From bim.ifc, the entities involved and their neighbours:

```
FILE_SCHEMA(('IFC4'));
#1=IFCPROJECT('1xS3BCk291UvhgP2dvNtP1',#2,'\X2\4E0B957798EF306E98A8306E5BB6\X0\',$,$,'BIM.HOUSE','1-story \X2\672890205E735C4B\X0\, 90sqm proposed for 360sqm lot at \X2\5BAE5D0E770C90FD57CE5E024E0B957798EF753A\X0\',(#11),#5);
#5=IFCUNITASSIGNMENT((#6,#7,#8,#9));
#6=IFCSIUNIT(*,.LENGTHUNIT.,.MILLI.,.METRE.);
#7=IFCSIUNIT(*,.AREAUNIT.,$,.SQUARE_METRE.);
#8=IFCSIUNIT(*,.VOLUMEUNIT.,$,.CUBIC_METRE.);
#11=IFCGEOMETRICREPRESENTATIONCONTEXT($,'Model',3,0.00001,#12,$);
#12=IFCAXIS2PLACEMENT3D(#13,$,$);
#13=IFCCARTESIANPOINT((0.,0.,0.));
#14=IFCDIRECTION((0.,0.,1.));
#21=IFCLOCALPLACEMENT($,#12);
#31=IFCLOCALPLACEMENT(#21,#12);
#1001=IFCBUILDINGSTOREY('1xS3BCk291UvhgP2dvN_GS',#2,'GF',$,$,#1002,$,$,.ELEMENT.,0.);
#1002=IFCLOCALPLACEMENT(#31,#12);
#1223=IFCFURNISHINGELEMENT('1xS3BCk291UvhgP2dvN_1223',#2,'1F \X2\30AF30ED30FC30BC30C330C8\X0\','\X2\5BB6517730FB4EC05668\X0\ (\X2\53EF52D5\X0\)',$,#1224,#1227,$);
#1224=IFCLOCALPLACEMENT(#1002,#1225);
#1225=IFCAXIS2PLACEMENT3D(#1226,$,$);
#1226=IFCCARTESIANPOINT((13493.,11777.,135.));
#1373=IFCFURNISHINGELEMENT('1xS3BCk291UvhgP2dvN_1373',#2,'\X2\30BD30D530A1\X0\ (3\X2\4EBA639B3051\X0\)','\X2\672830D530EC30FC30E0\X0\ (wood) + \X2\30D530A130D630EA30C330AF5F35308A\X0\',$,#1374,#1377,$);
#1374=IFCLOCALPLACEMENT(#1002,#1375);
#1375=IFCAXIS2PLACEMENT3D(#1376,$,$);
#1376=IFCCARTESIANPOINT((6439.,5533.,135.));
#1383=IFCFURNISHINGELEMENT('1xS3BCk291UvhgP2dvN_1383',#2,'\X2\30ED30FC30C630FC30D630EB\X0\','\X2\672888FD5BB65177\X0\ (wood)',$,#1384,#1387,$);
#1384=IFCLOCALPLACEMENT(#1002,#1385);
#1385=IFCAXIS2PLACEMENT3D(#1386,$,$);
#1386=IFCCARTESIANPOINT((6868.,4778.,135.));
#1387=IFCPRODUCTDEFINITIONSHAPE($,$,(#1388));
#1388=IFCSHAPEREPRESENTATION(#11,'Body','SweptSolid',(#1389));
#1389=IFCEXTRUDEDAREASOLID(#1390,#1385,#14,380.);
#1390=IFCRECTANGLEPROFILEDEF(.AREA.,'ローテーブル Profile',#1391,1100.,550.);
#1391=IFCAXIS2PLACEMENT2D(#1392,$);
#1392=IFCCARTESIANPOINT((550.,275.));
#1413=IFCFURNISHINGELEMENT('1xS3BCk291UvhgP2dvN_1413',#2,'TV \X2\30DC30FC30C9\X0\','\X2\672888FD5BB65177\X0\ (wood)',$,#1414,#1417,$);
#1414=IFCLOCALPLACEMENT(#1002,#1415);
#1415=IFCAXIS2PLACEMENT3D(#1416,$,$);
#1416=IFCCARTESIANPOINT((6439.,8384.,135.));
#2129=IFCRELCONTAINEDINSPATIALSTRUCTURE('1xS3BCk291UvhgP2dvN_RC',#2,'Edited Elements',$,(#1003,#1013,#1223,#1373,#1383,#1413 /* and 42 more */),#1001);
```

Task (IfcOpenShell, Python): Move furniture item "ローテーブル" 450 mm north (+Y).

```python
import ifcopenshell
import ifcopenshell.api.geometry
import ifcopenshell.util.placement
import ifcopenshell.util.unit

model = ifcopenshell.open("bim.ifc")
unit_scale = ifcopenshell.util.unit.calculate_unit_scale(model)

item = model.by_guid("1xS3BCk291UvhgP2dvN_1383")
matrix = ifcopenshell.util.placement.get_local_placement(item.ObjectPlacement)
matrix[1, 3] += 0.45 / unit_scale
ifcopenshell.api.geometry.edit_object_placement(model, product=item, matrix=matrix, is_si=False)

print(ifcopenshell.util.placement.get_local_placement(item.ObjectPlacement).round(3) + 0.0)

model.write("bim_updated.ifc")
```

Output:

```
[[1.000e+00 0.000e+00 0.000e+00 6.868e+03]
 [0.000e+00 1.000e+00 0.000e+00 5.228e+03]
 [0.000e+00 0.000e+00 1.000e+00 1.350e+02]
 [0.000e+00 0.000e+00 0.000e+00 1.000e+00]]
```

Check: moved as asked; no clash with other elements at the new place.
